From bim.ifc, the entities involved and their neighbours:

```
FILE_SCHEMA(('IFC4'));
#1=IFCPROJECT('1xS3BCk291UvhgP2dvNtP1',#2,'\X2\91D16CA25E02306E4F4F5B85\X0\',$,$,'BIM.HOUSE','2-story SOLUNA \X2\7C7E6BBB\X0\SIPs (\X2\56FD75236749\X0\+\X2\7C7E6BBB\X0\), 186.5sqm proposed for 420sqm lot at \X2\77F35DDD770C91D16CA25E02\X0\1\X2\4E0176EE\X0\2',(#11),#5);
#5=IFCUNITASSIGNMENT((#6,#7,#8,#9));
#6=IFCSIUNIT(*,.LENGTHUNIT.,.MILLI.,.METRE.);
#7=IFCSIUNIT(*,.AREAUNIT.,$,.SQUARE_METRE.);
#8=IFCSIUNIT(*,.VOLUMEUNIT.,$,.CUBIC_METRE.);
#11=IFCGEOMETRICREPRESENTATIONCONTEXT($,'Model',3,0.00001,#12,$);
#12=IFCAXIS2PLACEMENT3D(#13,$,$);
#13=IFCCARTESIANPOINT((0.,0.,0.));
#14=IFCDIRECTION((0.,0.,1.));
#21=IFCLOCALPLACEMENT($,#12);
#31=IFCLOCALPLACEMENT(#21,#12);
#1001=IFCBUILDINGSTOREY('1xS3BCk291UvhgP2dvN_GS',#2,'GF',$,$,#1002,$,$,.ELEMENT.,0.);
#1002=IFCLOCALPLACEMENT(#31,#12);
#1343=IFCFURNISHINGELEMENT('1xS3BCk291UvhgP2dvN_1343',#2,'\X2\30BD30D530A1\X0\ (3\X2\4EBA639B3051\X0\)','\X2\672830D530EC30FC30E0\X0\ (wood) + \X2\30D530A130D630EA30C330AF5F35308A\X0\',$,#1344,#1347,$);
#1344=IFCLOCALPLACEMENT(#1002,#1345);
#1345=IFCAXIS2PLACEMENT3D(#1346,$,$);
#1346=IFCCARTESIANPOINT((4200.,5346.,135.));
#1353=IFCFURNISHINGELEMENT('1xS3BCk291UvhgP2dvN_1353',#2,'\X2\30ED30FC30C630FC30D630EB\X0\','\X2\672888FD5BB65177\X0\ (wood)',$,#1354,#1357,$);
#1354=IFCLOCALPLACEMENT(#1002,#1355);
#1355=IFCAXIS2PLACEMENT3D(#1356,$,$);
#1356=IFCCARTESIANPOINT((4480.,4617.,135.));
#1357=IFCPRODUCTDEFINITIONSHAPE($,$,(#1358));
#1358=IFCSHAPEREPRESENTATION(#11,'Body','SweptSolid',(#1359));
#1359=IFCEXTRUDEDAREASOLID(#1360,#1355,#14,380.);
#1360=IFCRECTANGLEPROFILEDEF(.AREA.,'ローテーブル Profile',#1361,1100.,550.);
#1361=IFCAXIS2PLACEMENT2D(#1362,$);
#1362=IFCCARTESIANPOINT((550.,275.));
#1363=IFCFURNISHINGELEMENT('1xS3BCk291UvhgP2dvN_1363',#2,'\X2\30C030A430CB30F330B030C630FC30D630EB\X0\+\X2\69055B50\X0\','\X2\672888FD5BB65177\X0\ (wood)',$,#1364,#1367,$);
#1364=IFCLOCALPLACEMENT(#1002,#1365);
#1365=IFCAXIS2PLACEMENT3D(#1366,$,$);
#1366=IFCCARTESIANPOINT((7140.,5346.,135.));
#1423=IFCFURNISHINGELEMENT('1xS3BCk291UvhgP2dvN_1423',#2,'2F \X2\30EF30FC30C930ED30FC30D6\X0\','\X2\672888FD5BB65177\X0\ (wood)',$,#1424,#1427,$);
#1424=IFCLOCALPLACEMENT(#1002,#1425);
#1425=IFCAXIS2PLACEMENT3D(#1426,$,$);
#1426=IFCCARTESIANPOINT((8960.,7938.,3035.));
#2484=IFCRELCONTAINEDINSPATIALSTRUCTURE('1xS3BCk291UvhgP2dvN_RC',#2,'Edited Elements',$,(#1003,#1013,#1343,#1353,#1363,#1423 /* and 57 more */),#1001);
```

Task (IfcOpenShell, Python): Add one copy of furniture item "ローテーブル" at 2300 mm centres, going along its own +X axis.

```python
import ifcopenshell
import ifcopenshell.api.geometry
import ifcopenshell.api.root
import ifcopenshell.util.element
import ifcopenshell.util.placement
import ifcopenshell.util.unit

model = ifcopenshell.open("bim.ifc")
unit_scale = ifcopenshell.util.unit.calculate_unit_scale(model)


def reuse_history(source, copy):
    """copy_class also copies each property set's owner history, people and application; keep the originals."""
    for rel in copy.IsDefinedBy:
        if rel.is_a("IfcRelDefinesByProperties") and (history := rel.RelatingPropertyDefinition.OwnerHistory):
            rel.RelatingPropertyDefinition.OwnerHistory = source.OwnerHistory
            ifcopenshell.util.element.remove_deep2(model, history)


source = model.by_id(1353)
base = ifcopenshell.util.placement.get_local_placement(source.ObjectPlacement)
step = base[:3, 0] * 2.3 / unit_scale

for i in range(1, 2):
    copy = ifcopenshell.api.root.copy_class(model, product=source)
    copy.Representation = ifcopenshell.util.element.copy_deep(
        model, source.Representation, exclude=["IfcGeometricRepresentationContext", "IfcRepresentationMap"]
    )
    reuse_history(source, copy)
    matrix = base.copy()
    matrix[:3, 3] += i * step
    print("added at", matrix[:3, 3].round(3) + 0.0)
    ifcopenshell.api.geometry.edit_object_placement(model, product=copy, matrix=matrix, is_si=False)

model.write("bim_edited.ifc")
```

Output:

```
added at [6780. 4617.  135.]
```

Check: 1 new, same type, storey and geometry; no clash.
